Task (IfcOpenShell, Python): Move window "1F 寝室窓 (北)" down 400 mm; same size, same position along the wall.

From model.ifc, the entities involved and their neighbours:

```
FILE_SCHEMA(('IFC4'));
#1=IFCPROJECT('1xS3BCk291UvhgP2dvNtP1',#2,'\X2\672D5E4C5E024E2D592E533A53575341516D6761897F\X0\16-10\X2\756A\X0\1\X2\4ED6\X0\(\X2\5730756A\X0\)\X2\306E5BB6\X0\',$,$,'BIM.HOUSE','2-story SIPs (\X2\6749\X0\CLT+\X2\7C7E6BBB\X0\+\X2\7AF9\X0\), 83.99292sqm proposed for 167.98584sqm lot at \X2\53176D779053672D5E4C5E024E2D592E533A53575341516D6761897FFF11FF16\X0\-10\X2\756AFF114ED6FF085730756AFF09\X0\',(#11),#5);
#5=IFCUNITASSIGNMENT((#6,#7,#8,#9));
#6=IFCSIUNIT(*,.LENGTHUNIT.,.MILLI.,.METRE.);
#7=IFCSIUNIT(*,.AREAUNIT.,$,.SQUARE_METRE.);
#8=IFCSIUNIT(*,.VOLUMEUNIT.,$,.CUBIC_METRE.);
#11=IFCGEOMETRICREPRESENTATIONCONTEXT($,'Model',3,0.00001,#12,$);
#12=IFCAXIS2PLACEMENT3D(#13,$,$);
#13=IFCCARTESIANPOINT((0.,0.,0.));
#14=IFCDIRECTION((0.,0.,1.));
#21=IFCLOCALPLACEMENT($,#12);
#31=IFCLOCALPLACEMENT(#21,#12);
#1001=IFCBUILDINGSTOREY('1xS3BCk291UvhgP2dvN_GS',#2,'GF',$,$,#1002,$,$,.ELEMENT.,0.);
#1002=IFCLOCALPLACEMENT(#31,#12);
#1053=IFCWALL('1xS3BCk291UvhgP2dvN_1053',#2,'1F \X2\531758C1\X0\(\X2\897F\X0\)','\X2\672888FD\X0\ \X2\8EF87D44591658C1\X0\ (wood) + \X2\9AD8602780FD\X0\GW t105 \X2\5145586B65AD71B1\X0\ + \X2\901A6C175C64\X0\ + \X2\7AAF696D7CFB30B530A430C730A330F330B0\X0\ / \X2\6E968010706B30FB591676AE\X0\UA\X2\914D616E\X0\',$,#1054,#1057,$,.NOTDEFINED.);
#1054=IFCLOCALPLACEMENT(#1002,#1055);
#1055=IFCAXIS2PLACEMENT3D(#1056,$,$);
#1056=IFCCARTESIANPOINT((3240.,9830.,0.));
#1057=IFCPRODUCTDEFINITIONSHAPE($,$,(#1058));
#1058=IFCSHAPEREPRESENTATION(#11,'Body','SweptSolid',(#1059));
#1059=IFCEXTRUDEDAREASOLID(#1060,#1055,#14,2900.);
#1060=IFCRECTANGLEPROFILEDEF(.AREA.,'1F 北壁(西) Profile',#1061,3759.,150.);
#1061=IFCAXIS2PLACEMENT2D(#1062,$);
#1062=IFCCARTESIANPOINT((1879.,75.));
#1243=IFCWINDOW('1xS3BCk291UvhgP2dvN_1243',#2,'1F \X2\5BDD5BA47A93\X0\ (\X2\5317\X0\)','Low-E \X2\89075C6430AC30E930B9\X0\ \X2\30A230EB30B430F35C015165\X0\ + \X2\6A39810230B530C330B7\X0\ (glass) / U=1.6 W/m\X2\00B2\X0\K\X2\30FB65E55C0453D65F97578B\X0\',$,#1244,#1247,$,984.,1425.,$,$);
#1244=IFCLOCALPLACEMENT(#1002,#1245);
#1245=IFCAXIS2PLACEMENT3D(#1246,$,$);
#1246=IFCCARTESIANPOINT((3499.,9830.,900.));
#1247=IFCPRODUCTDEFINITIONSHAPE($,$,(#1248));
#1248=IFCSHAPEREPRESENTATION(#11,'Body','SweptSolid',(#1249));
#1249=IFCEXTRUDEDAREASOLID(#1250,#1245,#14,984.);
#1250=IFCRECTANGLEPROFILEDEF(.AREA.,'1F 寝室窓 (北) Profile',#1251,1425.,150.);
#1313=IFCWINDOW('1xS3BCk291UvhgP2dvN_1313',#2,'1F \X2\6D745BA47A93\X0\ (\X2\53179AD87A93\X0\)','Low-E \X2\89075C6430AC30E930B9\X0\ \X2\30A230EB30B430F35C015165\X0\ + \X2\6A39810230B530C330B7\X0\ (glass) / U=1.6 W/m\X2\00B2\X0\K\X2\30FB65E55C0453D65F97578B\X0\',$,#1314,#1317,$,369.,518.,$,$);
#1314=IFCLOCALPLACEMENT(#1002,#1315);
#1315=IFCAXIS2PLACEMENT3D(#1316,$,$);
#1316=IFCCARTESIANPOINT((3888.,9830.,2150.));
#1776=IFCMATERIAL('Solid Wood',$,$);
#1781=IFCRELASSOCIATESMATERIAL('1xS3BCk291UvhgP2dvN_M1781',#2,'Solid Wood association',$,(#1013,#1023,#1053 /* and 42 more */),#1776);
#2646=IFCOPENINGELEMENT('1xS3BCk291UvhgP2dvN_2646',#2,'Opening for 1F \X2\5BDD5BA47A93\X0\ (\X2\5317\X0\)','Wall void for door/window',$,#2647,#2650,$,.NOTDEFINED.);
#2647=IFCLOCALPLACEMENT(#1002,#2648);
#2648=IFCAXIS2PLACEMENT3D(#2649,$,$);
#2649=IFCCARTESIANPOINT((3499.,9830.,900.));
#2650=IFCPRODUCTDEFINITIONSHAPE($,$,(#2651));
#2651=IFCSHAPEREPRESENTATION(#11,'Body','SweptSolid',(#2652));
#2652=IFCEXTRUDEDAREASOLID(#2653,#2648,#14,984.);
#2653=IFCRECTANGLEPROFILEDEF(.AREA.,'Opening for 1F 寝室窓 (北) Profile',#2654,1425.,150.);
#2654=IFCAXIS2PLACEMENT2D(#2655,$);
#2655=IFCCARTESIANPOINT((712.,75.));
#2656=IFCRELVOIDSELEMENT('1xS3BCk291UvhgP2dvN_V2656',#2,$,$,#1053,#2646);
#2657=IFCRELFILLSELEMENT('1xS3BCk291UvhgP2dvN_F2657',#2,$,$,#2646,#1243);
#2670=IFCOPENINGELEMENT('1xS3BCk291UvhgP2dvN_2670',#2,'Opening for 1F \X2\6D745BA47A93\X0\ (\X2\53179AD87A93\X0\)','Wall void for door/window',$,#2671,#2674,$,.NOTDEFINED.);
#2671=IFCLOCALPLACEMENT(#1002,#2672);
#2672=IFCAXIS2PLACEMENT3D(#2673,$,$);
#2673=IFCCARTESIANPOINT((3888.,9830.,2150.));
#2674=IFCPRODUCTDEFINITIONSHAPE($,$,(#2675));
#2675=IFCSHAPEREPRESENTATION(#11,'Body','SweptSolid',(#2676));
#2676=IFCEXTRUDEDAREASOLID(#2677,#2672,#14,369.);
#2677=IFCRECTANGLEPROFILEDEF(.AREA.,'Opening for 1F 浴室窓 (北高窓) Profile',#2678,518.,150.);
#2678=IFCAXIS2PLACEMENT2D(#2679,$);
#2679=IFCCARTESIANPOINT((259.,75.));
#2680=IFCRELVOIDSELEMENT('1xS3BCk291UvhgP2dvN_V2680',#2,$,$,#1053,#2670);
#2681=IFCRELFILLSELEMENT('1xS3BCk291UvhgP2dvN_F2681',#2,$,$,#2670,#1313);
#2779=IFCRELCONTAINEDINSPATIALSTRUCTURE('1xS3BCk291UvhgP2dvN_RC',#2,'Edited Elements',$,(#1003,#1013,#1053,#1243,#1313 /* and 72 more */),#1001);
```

```python
import numpy as np
import ifcopenshell
import ifcopenshell.api.geometry
import ifcopenshell.util.placement
import ifcopenshell.util.unit

model = ifcopenshell.open("model.ifc")
unit_scale = ifcopenshell.util.unit.calculate_unit_scale(model)

window = model.by_guid("1xS3BCk291UvhgP2dvN_1243")
opening = window.FillsVoids[0].RelatingOpeningElement
dz = -0.4 / unit_scale

shift = np.array([0.0, 0.0, dz])
# The window is not placed relative to its opening, so move both.
for product in (opening, window):
    matrix = ifcopenshell.util.placement.get_local_placement(product.ObjectPlacement)
    matrix[:3, 3] += shift
    ifcopenshell.api.geometry.edit_object_placement(model, product=product, matrix=matrix, is_si=False)

print(f"moved by {dz * unit_scale:+.3f} m")

model.write("model_edited.ifc")
```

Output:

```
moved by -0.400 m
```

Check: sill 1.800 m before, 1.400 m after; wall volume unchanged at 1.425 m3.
